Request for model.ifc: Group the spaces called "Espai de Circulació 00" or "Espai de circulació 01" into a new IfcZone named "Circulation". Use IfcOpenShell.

First a look at what the model holds.

```python
import ifcopenshell

model = ifcopenshell.open("model.ifc")
print(model.schema)
seen = {}
for space in model.by_type("IfcSpace"):
    seen[space.LongName] = seen.get(space.LongName, 0) + 1
for name, count in sorted(seen.items(), key=str):
    print(count, "x", name)
print("zones:", [z.Name for z in model.by_type("IfcZone")][:20])
```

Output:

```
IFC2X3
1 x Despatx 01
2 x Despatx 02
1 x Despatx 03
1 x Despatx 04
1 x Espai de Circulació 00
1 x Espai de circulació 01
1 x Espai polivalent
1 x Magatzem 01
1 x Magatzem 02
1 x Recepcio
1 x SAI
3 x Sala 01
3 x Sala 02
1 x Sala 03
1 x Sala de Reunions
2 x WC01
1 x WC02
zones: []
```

```python
import ifcopenshell
import ifcopenshell.api.group
import ifcopenshell.api.root

model = ifcopenshell.open("model.ifc")

names = {"Espai de Circulació 00", "Espai de circulació 01"}
spaces = [s for s in model.by_type("IfcSpace") if s.LongName in names]

zone = ifcopenshell.api.root.create_entity(model, ifc_class="IfcZone", name="Circulation")
ifcopenshell.api.group.assign_group(model, products=spaces, group=zone)
print(len(spaces), "spaces in", zone.Name)

model.write("model_rev.ifc")
```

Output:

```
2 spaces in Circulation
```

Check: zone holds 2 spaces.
